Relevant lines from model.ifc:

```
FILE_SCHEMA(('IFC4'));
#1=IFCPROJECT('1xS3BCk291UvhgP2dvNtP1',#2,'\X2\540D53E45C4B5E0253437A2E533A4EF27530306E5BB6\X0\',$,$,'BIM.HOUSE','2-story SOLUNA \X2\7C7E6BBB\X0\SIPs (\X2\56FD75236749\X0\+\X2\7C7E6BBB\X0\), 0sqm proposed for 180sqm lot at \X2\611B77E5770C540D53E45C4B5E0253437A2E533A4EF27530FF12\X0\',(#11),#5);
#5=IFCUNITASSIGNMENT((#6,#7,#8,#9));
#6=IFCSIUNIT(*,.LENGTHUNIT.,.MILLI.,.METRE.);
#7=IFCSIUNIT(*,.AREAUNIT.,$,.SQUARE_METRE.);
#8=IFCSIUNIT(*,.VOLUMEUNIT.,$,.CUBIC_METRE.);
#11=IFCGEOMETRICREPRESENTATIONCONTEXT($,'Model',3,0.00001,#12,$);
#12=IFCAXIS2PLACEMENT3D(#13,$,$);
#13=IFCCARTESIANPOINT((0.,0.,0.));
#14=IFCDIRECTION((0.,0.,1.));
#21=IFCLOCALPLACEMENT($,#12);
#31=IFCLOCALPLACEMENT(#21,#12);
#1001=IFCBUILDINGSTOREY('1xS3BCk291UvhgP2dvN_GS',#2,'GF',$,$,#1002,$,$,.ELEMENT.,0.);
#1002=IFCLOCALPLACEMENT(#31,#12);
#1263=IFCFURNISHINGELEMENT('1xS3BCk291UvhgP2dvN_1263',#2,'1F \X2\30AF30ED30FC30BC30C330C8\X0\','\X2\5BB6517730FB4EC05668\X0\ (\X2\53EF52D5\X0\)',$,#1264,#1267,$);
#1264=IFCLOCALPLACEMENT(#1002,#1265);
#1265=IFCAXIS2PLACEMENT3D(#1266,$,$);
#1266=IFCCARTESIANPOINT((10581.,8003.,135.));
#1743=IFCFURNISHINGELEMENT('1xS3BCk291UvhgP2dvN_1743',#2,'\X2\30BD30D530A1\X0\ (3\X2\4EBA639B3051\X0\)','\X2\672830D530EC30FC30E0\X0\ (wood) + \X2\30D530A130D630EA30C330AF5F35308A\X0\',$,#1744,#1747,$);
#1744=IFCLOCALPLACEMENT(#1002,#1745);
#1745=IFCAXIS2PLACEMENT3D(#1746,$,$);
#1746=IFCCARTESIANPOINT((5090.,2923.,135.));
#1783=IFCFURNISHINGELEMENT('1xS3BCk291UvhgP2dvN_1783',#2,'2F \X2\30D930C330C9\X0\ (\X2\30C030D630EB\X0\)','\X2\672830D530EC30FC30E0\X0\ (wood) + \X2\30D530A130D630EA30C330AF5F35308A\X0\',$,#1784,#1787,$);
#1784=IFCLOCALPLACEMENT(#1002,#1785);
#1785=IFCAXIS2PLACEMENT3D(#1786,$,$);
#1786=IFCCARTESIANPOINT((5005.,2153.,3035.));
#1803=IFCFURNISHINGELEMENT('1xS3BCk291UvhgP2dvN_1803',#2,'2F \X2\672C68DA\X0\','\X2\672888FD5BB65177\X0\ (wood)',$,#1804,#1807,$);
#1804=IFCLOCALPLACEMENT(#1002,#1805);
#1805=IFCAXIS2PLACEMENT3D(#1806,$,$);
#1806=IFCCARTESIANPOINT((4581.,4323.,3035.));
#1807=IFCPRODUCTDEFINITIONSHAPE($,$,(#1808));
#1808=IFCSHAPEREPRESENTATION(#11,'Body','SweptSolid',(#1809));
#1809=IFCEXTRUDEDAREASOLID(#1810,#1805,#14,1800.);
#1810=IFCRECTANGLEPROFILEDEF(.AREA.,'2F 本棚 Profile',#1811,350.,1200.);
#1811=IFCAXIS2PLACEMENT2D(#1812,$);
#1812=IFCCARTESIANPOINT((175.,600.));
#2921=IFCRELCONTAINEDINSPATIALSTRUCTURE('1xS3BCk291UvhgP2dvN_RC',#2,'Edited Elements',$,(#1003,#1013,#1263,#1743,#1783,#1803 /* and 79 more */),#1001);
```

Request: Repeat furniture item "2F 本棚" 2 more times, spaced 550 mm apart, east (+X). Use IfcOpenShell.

```python
import numpy as np
import ifcopenshell
import ifcopenshell.api.geometry
import ifcopenshell.api.root
import ifcopenshell.util.element
import ifcopenshell.util.placement
import ifcopenshell.util.unit

model = ifcopenshell.open("model.ifc")
unit_scale = ifcopenshell.util.unit.calculate_unit_scale(model)


def reuse_history(source, copy):
    """copy_class also copies each property set's owner history, people and application; keep the originals."""
    for rel in copy.IsDefinedBy:
        if rel.is_a("IfcRelDefinesByProperties") and (history := rel.RelatingPropertyDefinition.OwnerHistory):
            rel.RelatingPropertyDefinition.OwnerHistory = source.OwnerHistory
            ifcopenshell.util.element.remove_deep2(model, history)


source = model.by_guid("1xS3BCk291UvhgP2dvN_1803")
base = ifcopenshell.util.placement.get_local_placement(source.ObjectPlacement)
step = np.array([1.0, 0.0, 0.0]) * 0.55 / unit_scale

for i in range(1, 3):
    copy = ifcopenshell.api.root.copy_class(model, product=source)
    copy.Representation = ifcopenshell.util.element.copy_deep(
        model, source.Representation, exclude=["IfcGeometricRepresentationContext", "IfcRepresentationMap"]
    )
    reuse_history(source, copy)
    matrix = base.copy()
    matrix[:3, 3] += i * step
    print("added at", matrix[:3, 3].round(3) + 0.0)
    ifcopenshell.api.geometry.edit_object_placement(model, product=copy, matrix=matrix, is_si=False)

model.write("model_rev.ifc")
```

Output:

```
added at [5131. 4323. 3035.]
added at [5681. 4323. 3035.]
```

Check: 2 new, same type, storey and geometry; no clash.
